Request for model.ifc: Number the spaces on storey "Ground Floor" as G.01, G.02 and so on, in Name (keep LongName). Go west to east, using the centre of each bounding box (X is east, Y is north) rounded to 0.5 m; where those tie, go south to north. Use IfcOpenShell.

First a look at what the model holds.

```python
import ifcopenshell
import ifcopenshell.util.element
import ifcopenshell.util.placement

model = ifcopenshell.open("model.ifc")
print(model.schema)
storey = next(s for s in model.by_type("IfcBuildingStorey") if s.Name == "Ground Floor")
spaces = [e for e in ifcopenshell.util.element.get_decomposition(storey) if e.is_a("IfcSpace")]
for e in sorted(spaces, key=lambda e: e.id()):
    origin = ifcopenshell.util.placement.get_local_placement(e.ObjectPlacement)[:3, 3]
    print(e.id(), e.Name, e.LongName, origin.round(2) + 0.0, sep=" | ")
```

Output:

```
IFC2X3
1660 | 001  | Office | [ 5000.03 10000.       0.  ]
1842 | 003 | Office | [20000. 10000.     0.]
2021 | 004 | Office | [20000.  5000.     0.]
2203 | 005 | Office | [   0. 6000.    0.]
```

```python
import ifcopenshell
import ifcopenshell.geom
import ifcopenshell.util.element
import ifcopenshell.util.shape

model = ifcopenshell.open("model.ifc")
settings = ifcopenshell.geom.settings()
settings.set("use-world-coords", True)


def centre(element):
    shape = ifcopenshell.geom.create_shape(settings, element)
    return ifcopenshell.util.shape.get_bbox_centroid(shape.geometry)


storey = next(s for s in model.by_type("IfcBuildingStorey") if s.Name == "Ground Floor")
spaces = [e for e in ifcopenshell.util.element.get_decomposition(storey) if e.is_a("IfcSpace")]

# Insertion points can sit at a corner or the storey origin, so sort by the geometry (in metres).
centres = {e: centre(e) for e in spaces}
spaces.sort(key=lambda e: (round(centres[e][0] / 0.5), centres[e][1]))

for i, e in enumerate(spaces, start=1):
    number = f"G.{i:02d}"
    e.Name = number
    print(e.id(), number)

model.write("model_v2.ifc")
```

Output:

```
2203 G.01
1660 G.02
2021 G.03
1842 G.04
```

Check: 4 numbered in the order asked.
